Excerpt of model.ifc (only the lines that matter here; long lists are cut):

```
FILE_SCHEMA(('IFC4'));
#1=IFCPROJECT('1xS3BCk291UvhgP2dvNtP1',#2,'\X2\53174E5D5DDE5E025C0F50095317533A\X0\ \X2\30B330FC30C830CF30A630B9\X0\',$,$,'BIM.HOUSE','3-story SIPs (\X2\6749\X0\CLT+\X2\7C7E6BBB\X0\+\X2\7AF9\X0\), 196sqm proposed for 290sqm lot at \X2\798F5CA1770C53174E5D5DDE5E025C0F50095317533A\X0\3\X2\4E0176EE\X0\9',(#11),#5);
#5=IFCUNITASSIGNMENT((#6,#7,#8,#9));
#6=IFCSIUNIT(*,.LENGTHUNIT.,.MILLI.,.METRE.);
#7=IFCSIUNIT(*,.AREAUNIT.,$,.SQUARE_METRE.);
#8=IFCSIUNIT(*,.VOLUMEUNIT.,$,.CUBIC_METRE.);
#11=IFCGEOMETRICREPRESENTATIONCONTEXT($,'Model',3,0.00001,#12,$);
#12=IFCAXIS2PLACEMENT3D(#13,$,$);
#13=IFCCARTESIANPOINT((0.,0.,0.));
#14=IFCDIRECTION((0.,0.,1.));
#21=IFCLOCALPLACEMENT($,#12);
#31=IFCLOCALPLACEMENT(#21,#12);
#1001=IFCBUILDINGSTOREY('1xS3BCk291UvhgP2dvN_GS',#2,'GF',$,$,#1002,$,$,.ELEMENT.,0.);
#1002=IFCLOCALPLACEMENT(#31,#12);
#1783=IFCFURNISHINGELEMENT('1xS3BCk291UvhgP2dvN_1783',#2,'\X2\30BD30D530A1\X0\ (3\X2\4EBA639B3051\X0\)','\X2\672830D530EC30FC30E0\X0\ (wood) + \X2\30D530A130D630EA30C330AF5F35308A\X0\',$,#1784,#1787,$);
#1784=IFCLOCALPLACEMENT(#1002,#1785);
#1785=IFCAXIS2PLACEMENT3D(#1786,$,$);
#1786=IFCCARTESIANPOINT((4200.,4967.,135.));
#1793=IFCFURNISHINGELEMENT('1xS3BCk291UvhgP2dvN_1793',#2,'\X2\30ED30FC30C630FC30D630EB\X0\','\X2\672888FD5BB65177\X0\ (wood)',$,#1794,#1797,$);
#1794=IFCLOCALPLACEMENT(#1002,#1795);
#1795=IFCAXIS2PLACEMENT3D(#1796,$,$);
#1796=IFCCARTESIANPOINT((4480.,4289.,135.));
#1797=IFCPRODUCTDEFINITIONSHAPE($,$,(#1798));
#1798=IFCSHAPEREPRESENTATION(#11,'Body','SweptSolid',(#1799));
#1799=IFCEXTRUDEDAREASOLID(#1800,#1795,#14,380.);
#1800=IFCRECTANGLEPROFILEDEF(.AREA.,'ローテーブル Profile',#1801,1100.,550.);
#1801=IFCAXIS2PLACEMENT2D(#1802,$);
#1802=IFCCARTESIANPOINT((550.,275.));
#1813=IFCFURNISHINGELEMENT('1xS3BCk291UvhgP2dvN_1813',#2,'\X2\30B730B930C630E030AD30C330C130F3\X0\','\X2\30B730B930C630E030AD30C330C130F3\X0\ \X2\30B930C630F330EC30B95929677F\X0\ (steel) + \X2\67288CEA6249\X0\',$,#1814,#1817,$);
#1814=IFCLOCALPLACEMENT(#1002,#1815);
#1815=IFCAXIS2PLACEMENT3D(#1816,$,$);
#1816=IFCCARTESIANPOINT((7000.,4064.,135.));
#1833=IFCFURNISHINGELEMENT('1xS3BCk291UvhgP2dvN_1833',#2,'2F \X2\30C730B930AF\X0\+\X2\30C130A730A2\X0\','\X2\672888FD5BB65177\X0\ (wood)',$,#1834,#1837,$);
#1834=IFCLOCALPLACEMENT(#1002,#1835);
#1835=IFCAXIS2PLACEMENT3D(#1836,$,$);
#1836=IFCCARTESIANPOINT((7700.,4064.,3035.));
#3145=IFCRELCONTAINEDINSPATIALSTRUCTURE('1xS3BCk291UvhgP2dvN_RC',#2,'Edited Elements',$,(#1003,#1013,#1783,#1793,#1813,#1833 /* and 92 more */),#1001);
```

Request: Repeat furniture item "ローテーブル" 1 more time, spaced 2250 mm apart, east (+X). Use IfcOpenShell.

```python
import numpy as np
import ifcopenshell
import ifcopenshell.api.geometry
import ifcopenshell.api.root
import ifcopenshell.util.element
import ifcopenshell.util.placement

model = ifcopenshell.open("model.ifc")


def reuse_history(source, copy):
    """copy_class also copies each property set's owner history, people and application; keep the originals."""
    for rel in copy.IsDefinedBy:
        if rel.is_a("IfcRelDefinesByProperties") and (history := rel.RelatingPropertyDefinition.OwnerHistory):
            rel.RelatingPropertyDefinition.OwnerHistory = source.OwnerHistory
            ifcopenshell.util.element.remove_deep2(model, history)


source = model.by_id(1793)
base = ifcopenshell.util.placement.get_local_placement(source.ObjectPlacement)
step = np.array([1.0, 0.0, 0.0]) * 2250.0

for i in range(1, 2):
    copy = ifcopenshell.api.root.copy_class(model, product=source)
    copy.Representation = ifcopenshell.util.element.copy_deep(
        model, source.Representation, exclude=["IfcGeometricRepresentationContext", "IfcRepresentationMap"]
    )
    reuse_history(source, copy)
    matrix = base.copy()
    matrix[:3, 3] += i * step
    print("added at", matrix[:3, 3].round(3) + 0.0)
    ifcopenshell.api.geometry.edit_object_placement(model, product=copy, matrix=matrix, is_si=False)

model.write("model_updated.ifc")
```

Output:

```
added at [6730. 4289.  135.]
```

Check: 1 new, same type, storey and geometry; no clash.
